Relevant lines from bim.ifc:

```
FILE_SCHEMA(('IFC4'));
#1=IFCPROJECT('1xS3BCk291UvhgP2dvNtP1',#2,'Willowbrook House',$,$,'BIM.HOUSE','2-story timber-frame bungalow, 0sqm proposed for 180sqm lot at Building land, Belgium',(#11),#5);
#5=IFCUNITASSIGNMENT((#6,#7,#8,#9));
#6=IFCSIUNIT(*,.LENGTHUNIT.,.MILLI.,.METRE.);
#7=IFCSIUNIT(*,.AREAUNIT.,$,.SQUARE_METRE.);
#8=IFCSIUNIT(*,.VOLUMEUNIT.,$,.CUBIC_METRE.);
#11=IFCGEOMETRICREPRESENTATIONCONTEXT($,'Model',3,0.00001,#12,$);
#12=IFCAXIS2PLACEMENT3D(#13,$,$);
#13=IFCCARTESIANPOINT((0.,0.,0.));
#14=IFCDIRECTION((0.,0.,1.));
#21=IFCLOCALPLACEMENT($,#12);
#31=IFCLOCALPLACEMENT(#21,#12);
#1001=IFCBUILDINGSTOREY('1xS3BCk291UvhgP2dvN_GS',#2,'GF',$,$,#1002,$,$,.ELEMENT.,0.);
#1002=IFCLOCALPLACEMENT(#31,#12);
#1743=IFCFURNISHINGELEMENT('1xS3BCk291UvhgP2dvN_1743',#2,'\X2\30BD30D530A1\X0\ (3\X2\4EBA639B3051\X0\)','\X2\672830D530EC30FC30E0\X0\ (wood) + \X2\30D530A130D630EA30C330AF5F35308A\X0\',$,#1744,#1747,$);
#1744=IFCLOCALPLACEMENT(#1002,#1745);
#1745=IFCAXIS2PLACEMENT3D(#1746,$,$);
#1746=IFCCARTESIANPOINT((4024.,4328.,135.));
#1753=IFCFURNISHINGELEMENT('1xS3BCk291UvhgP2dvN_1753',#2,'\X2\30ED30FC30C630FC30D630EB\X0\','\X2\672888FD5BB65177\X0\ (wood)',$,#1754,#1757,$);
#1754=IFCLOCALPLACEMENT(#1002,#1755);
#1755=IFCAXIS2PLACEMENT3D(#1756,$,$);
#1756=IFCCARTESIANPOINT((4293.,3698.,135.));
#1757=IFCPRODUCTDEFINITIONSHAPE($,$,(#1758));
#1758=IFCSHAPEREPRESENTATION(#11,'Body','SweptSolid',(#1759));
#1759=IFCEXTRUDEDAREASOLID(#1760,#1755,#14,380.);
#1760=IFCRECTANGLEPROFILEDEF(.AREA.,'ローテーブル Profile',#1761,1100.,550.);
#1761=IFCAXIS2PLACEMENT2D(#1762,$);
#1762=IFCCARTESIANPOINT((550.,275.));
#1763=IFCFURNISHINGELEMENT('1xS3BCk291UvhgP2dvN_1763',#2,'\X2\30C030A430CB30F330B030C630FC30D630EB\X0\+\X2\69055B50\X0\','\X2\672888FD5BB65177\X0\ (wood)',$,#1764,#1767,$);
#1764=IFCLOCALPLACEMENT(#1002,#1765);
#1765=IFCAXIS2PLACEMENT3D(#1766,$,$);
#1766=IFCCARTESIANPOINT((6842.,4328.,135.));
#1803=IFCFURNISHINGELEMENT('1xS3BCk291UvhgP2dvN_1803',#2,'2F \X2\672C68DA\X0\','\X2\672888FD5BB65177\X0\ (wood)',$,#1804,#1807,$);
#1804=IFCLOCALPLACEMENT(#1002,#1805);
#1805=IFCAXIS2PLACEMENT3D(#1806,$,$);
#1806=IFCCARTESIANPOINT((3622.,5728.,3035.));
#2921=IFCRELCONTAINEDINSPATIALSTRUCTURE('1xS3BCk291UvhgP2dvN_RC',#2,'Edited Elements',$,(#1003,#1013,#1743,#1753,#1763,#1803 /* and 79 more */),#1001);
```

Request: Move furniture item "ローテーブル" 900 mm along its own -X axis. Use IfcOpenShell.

```python
import ifcopenshell
import ifcopenshell.api.geometry
import ifcopenshell.util.placement
import ifcopenshell.util.unit

model = ifcopenshell.open("bim.ifc")
unit_scale = ifcopenshell.util.unit.calculate_unit_scale(model)

item = model.by_id(1753)
matrix = ifcopenshell.util.placement.get_local_placement(item.ObjectPlacement)
matrix[:3, 3] -= matrix[:3, 0] * 0.9 / unit_scale
ifcopenshell.api.geometry.edit_object_placement(model, product=item, matrix=matrix, is_si=False)

print(ifcopenshell.util.placement.get_local_placement(item.ObjectPlacement).round(3) + 0.0)

model.write("bim_v2.ifc")
```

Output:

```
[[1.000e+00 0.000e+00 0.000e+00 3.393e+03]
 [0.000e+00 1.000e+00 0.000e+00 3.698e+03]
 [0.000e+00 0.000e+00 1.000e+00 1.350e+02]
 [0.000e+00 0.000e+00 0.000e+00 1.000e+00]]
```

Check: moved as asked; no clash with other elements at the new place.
